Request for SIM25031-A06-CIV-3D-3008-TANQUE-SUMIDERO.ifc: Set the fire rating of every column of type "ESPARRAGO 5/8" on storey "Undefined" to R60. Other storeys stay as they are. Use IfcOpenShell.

First a look at what the model holds.

```python
import ifcopenshell
import ifcopenshell.util.element

model = ifcopenshell.open("SIM25031-A06-CIV-3D-3008-TANQUE-SUMIDERO.ifc")
print(model.schema)
storey = next(s for s in model.by_type("IfcBuildingStorey") if s.Name == "Undefined")
columns = [e for e in ifcopenshell.util.element.get_decomposition(storey) if e.is_a("IfcColumn")]
seen = {}
for e in columns:
    element_type = ifcopenshell.util.element.get_type(e)
    key = (element_type.Name if element_type != e and element_type else None, ifcopenshell.util.element.get_pset(e, "Pset_ColumnCommon", "FireRating"))
    seen[key] = seen.get(key, 0) + 1
for (name, value), count in sorted(seen.items(), key=str):
    print(count, "x", name, "|", value)
```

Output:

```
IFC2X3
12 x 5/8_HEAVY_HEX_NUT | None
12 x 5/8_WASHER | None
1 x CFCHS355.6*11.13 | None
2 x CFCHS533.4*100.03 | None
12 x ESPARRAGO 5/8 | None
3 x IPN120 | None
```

```python
import ifcopenshell
import ifcopenshell.api.pset
import ifcopenshell.util.element

model = ifcopenshell.open("SIM25031-A06-CIV-3D-3008-TANQUE-SUMIDERO.ifc")

storey = next(s for s in model.by_type("IfcBuildingStorey") if s.Name == "Undefined")
columns = [e for e in ifcopenshell.util.element.get_decomposition(storey) if e.is_a("IfcColumn")]

count = 0
for e in columns:
    element_type = ifcopenshell.util.element.get_type(e)
    if element_type in (None, e) or element_type.Name != "ESPARRAGO 5/8":
        continue
    found = ifcopenshell.util.element.get_pset(e, "Pset_ColumnCommon", should_inherit=False)
    if found:
        pset = model.by_id(found["id"])
        if len(ifcopenshell.util.element.get_elements_by_pset(pset)) > 1:
            pset = ifcopenshell.api.pset.unshare_pset(model, products=[e], pset=pset)[0]
    else:
        pset = ifcopenshell.api.pset.add_pset(model, product=e, name="Pset_ColumnCommon")
    ifcopenshell.api.pset.edit_pset(model, pset=pset, properties={"FireRating": "R60"})
    count += 1

print(count, "columns updated")

model.write("SIM25031-A06-CIV-3D-3008-TANQUE-SUMIDERO-out.ifc")
```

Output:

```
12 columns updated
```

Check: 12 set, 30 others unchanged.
